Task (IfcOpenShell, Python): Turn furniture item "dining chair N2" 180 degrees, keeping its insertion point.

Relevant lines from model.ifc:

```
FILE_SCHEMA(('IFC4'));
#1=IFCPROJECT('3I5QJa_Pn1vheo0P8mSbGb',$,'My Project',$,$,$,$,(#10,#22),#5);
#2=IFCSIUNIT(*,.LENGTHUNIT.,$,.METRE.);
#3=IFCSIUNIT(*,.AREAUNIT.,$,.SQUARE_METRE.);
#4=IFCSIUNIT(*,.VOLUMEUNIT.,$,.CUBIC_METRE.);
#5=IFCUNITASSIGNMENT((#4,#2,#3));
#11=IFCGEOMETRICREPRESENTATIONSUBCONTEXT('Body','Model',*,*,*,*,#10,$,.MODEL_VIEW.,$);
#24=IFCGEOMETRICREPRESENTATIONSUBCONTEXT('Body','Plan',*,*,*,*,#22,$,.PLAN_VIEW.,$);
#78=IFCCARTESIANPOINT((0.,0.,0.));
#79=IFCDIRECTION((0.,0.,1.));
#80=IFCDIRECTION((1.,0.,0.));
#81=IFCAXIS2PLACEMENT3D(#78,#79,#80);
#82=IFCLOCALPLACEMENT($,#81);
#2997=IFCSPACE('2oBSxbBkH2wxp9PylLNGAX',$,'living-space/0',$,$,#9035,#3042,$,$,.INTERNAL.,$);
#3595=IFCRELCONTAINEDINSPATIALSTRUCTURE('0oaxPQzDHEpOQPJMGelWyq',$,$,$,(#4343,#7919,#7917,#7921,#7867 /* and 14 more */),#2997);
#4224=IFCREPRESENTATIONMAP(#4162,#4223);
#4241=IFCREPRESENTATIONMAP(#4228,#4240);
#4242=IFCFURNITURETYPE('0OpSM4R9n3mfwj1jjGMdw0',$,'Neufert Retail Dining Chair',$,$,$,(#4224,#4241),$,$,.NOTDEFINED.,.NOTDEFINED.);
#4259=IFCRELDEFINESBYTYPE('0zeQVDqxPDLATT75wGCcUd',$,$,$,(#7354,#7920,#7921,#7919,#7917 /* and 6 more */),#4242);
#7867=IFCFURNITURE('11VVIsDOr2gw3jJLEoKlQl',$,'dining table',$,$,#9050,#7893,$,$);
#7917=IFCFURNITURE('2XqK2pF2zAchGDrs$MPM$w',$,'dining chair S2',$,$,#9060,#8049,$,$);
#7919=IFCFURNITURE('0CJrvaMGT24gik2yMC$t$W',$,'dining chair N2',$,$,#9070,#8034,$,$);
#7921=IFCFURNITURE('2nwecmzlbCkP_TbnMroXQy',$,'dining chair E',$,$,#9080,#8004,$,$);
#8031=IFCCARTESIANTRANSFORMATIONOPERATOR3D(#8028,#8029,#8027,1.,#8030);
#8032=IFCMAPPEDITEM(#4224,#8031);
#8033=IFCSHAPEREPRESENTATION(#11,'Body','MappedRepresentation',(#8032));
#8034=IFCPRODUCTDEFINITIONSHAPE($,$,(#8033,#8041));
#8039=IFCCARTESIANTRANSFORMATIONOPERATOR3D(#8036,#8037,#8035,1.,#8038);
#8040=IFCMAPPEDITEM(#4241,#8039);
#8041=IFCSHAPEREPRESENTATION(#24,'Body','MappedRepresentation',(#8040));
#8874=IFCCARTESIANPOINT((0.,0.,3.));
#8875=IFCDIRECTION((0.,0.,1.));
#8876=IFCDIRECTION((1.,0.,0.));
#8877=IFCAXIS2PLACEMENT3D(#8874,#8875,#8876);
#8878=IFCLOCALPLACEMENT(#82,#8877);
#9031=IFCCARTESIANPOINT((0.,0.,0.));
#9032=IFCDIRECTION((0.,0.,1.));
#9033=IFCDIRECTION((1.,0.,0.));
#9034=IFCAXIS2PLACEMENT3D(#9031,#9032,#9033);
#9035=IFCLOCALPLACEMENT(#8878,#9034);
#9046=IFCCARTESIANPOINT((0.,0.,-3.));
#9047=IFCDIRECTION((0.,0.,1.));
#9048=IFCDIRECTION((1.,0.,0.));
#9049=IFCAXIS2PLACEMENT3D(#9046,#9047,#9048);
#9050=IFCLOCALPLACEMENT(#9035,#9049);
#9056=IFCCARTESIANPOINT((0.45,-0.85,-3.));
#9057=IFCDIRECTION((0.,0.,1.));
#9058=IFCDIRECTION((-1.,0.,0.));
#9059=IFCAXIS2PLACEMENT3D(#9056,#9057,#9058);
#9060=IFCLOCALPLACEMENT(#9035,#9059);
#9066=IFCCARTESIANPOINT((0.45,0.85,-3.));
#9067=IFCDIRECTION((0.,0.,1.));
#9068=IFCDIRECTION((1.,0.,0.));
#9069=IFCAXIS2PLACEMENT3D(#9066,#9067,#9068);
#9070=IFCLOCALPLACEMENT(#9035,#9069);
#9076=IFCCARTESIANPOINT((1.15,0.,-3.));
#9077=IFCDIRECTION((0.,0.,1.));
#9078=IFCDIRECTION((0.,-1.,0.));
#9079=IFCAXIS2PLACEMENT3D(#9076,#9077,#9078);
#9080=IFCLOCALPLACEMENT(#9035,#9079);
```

```python
import ifcopenshell
import ifcopenshell.api.geometry
import ifcopenshell.util.placement

model = ifcopenshell.open("model.ifc")

item = model.by_guid("0CJrvaMGT24gik2yMC$t$W")
matrix = ifcopenshell.util.placement.get_local_placement(item.ObjectPlacement)
matrix = matrix @ ifcopenshell.util.placement.rotation(180, "Z")
ifcopenshell.api.geometry.edit_object_placement(model, product=item, matrix=matrix, is_si=False)

print(ifcopenshell.util.placement.get_local_placement(item.ObjectPlacement).round(3) + 0.0)

model.write("model_edited.ifc")
```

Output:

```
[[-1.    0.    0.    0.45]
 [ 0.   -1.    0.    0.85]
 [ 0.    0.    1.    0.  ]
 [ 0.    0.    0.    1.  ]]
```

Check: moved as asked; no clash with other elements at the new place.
